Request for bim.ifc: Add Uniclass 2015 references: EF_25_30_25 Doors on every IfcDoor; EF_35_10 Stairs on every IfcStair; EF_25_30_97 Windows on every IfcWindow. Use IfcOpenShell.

First a look at what the model holds.

```python
import ifcopenshell

model = ifcopenshell.open("bim.ifc")
print(model.schema)
print("classifications:", [c.Name for c in model.by_type("IfcClassification")])
for ifc_class in ("IfcDoor", "IfcRoof", "IfcStair", "IfcWall", "IfcWindow"):
    print(ifc_class, len(model.by_type(ifc_class)))
```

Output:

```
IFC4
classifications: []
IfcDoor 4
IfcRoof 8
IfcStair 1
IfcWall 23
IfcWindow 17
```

```python
import ifcopenshell
import ifcopenshell.api.classification

model = ifcopenshell.open("bim.ifc")

system = ifcopenshell.api.classification.add_classification(model, classification="Uniclass 2015")

codes = {
    "IfcDoor": ("EF_25_30_25", "Doors"),
    "IfcStair": ("EF_35_10", "Stairs"),
    "IfcWindow": ("EF_25_30_97", "Windows"),
}
for ifc_class, (code, name) in codes.items():
    products = model.by_type(ifc_class)
    ifcopenshell.api.classification.add_reference(
        model, products=products, classification=system, identification=code, name=name
    )
    print(code, len(products))

model.write("bim_updated.ifc")
```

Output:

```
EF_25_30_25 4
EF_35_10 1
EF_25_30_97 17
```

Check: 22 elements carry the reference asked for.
